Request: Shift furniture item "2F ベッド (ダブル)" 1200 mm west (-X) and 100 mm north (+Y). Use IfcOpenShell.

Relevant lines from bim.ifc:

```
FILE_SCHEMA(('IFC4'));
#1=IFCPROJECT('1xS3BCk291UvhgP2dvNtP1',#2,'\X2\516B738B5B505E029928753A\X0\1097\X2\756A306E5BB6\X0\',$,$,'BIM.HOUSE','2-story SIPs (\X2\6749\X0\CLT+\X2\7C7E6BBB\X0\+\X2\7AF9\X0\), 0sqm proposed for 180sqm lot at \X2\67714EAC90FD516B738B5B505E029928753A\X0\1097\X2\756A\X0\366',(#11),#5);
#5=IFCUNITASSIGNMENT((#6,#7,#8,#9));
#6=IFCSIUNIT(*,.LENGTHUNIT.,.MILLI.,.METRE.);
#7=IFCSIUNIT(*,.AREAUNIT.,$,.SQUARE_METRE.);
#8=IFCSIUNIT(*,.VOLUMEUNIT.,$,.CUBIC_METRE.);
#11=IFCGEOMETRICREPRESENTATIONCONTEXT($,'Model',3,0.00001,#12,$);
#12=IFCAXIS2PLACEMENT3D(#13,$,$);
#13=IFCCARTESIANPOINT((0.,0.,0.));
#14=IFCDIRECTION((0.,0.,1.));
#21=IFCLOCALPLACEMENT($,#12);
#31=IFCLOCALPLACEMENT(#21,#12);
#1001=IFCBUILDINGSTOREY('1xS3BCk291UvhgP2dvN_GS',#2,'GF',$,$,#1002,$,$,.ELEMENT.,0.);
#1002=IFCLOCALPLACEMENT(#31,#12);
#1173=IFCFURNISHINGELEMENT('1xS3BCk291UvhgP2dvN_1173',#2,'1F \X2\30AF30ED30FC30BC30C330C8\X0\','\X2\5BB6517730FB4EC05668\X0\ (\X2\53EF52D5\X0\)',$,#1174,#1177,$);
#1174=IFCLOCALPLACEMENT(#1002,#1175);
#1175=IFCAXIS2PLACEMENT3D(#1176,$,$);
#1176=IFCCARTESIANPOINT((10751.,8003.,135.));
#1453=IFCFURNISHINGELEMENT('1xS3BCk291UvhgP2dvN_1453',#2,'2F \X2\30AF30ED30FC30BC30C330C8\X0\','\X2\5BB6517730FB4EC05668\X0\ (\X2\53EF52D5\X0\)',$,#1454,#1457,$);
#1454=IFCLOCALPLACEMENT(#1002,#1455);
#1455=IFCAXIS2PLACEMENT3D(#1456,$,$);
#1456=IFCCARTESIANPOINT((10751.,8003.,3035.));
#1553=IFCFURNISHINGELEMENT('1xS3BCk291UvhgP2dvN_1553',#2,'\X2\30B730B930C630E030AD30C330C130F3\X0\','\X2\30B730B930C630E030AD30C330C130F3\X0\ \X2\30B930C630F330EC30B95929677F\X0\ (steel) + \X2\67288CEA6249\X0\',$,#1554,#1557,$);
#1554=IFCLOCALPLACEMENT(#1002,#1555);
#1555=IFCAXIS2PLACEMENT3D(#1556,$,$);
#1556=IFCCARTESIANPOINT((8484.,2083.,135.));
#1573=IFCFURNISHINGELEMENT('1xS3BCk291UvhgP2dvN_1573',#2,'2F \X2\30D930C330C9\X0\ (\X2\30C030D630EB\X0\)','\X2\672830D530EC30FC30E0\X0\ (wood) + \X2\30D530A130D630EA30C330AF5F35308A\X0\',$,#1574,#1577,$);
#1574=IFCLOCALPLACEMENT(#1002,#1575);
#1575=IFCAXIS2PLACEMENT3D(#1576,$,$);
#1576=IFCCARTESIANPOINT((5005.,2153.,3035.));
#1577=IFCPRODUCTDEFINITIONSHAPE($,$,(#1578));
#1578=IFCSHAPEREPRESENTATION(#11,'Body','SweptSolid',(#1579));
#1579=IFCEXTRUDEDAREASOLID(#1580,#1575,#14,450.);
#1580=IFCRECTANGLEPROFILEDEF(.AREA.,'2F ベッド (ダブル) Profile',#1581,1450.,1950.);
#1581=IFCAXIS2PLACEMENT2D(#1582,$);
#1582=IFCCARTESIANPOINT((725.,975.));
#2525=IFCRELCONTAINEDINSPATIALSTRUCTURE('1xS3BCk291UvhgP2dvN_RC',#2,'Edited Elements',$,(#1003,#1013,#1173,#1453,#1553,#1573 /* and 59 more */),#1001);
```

```python
import ifcopenshell
import ifcopenshell.api.geometry
import ifcopenshell.util.placement
import ifcopenshell.util.unit

model = ifcopenshell.open("bim.ifc")
unit_scale = ifcopenshell.util.unit.calculate_unit_scale(model)

item = model.by_guid("1xS3BCk291UvhgP2dvN_1573")
matrix = ifcopenshell.util.placement.get_local_placement(item.ObjectPlacement)
matrix[0, 3] -= 1.2 / unit_scale
matrix[1, 3] += 0.1 / unit_scale
ifcopenshell.api.geometry.edit_object_placement(model, product=item, matrix=matrix, is_si=False)

print(ifcopenshell.util.placement.get_local_placement(item.ObjectPlacement).round(3) + 0.0)

model.write("bim_rev.ifc")
```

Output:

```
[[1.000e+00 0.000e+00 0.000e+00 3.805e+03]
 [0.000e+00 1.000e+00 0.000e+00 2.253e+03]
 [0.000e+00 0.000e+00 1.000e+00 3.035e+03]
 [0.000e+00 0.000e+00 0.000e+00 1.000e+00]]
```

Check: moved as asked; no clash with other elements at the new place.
